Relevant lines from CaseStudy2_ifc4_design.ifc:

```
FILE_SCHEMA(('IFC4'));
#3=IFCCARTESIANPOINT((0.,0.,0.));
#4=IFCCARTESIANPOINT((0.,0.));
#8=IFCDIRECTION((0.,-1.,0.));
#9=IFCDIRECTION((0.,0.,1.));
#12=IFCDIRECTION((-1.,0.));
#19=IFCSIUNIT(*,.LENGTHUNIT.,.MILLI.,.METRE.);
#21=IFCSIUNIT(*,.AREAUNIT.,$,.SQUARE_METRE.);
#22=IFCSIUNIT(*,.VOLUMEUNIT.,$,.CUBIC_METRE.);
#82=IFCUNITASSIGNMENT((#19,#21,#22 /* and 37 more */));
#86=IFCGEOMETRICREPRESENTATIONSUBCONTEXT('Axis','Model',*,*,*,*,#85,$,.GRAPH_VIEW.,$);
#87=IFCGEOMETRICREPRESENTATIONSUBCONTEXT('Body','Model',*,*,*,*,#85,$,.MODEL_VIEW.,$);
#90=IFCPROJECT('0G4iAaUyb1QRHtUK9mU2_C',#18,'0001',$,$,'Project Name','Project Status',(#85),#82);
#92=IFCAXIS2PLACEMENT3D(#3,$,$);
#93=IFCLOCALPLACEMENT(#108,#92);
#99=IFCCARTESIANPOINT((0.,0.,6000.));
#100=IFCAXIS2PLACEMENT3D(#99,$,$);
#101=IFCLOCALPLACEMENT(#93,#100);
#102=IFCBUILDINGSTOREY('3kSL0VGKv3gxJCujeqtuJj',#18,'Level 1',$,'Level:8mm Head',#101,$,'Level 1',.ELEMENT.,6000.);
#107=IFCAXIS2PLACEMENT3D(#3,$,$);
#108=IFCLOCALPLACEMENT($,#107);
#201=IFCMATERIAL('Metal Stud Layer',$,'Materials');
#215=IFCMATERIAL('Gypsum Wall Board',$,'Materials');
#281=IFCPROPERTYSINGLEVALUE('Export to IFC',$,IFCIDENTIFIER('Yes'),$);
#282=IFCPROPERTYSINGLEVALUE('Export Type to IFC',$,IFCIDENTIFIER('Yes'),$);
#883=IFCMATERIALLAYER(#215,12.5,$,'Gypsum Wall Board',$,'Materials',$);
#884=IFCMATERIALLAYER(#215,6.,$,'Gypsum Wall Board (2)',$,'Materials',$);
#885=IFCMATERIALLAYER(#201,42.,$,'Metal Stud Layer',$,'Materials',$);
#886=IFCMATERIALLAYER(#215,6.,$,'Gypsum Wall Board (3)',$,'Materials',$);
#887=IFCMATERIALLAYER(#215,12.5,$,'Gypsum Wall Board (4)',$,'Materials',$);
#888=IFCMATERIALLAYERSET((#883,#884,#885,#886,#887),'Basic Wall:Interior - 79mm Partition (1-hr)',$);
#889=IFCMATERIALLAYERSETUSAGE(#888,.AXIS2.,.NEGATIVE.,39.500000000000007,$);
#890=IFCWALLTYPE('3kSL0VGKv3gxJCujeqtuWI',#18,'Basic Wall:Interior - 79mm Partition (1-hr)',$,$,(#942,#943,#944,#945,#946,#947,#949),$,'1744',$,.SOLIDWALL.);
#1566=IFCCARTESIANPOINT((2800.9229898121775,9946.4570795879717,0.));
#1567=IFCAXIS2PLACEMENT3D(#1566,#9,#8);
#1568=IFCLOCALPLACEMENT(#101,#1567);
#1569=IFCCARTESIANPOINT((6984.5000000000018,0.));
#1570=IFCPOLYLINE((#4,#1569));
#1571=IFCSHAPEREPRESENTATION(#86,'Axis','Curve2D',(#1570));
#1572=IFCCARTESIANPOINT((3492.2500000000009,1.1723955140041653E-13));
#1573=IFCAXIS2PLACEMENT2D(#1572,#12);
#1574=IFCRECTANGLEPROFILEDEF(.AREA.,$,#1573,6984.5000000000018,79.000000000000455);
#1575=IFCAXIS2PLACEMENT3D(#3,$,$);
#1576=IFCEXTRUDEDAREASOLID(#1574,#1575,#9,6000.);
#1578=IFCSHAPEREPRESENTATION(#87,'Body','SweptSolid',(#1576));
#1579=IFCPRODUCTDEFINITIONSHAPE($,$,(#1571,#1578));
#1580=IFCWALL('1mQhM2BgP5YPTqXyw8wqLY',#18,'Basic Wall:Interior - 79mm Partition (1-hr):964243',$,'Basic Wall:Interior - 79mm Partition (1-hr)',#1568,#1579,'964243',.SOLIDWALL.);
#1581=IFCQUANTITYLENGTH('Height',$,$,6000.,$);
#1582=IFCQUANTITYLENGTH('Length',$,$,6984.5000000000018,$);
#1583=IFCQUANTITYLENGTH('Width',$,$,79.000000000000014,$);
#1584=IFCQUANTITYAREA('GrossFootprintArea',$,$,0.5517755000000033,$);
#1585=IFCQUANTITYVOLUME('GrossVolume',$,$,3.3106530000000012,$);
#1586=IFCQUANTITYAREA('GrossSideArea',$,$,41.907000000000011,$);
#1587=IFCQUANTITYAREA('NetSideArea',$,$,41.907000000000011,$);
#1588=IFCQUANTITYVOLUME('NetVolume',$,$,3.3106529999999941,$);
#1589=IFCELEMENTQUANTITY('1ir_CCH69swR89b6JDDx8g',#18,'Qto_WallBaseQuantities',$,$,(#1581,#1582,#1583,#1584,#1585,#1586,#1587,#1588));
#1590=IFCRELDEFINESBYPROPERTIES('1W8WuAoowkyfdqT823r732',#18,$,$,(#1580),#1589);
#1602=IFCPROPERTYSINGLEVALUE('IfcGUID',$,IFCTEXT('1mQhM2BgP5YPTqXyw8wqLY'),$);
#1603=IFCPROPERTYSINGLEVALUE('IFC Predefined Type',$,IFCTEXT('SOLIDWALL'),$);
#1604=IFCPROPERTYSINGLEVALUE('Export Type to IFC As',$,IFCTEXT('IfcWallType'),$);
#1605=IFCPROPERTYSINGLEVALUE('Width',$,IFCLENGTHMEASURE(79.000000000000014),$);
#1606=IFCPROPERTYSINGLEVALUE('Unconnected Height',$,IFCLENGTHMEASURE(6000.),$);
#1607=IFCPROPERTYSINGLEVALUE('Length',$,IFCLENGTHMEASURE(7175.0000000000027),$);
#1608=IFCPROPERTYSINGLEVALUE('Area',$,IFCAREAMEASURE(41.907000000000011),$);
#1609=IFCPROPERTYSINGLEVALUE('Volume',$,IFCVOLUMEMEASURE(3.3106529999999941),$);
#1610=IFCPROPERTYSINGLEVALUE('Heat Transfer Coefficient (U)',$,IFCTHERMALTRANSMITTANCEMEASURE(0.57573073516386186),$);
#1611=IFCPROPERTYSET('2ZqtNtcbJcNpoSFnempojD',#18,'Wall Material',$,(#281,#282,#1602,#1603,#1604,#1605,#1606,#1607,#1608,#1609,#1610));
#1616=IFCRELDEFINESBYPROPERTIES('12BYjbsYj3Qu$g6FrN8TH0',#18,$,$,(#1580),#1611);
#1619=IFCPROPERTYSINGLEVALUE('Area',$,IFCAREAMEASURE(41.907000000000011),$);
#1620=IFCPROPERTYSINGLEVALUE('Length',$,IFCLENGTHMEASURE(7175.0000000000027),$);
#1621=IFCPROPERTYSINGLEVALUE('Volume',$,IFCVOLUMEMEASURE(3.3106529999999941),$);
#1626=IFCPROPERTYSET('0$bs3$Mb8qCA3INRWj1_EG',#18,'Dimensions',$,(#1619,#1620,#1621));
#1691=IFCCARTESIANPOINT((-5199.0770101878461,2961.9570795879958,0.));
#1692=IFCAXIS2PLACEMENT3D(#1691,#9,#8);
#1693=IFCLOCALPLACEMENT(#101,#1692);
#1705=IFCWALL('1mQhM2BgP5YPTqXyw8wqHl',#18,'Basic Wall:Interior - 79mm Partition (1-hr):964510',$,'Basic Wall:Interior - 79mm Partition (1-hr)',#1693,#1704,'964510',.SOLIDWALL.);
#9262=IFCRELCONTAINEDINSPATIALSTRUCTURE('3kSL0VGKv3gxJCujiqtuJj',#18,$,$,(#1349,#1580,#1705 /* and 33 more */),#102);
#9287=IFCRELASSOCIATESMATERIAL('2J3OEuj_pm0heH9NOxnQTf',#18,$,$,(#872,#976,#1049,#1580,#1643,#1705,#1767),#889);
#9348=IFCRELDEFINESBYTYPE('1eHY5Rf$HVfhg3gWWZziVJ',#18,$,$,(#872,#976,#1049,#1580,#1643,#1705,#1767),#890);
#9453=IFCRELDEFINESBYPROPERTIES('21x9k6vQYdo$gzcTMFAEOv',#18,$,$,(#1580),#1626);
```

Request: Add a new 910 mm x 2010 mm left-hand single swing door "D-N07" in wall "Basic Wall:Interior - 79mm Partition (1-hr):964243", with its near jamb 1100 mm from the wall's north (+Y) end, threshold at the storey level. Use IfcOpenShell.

```python
import numpy as np
import ifcopenshell
import ifcopenshell.api.feature
import ifcopenshell.api.geometry
import ifcopenshell.api.pset
import ifcopenshell.api.root
import ifcopenshell.api.spatial
import ifcopenshell.geom
import ifcopenshell.util.element
import ifcopenshell.util.placement
import ifcopenshell.util.representation
import ifcopenshell.util.shape
import ifcopenshell.util.unit

model = ifcopenshell.open("CaseStudy2_ifc4_design.ifc")
unit_scale = ifcopenshell.util.unit.calculate_unit_scale(model)
area_scale = ifcopenshell.util.unit.calculate_unit_scale(model, "AREAUNIT")
volume_scale = ifcopenshell.util.unit.calculate_unit_scale(model, "VOLUMEUNIT")
settings = ifcopenshell.geom.settings()


def volume(element):
    """Net volume in cubic metres, openings subtracted."""
    shape = ifcopenshell.geom.create_shape(settings, element)
    return ifcopenshell.util.shape.get_volume(shape.geometry)


wall = model.by_guid("1mQhM2BgP5YPTqXyw8wqLY")
storey = ifcopenshell.util.element.get_container(wall, ifc_class="IfcBuildingStorey")
context = ifcopenshell.util.representation.get_context(model, "Model", "Body", "MODEL_VIEW")
before = volume(wall)

width, height, from_end, sill = 0.91, 2.01, 1.1, 0.0  # metres

# The wall runs along its own X axis, and the end named is its -X end.
wall_shape = ifcopenshell.geom.create_shape(settings, wall)
x, y, z = ifcopenshell.util.shape.get_vertices(wall_shape.geometry).T
start = x.min() + from_end
face, thickness = float(y.min()), float(y.max() - y.min())
wall_matrix = ifcopenshell.util.placement.get_local_placement(wall.ObjectPlacement)
level = ifcopenshell.util.placement.get_local_placement(storey.ObjectPlacement)[2, 3]


def in_wall(x, y):
    """Placement at x, y metres in the wall's axes, at sill height."""
    matrix = wall_matrix.copy()
    matrix[:, 3] = wall_matrix @ np.array([x / unit_scale, y / unit_scale, 0.0, 1.0])
    matrix[2, 3] = level + sill / unit_scale
    return matrix


# Opening: a box that overshoots both wall faces by 50 mm.
opening = ifcopenshell.api.root.create_entity(model, ifc_class="IfcOpeningElement", predefined_type="OPENING")
box = ifcopenshell.api.geometry.add_wall_representation(
    model, context=context, length=width, height=height, thickness=thickness + 0.1
)
ifcopenshell.api.geometry.assign_representation(model, product=opening, representation=box)
ifcopenshell.api.geometry.edit_object_placement(model, product=opening, matrix=in_wall(start, face - 0.05), is_si=False)
ifcopenshell.api.feature.add_feature(model, feature=opening, element=wall)

door = ifcopenshell.api.root.create_entity(model, ifc_class="IfcDoor", name="D-N07", predefined_type="DOOR")
door.OverallWidth, door.OverallHeight = width / unit_scale, height / unit_scale
door.OperationType = "SINGLE_SWING_LEFT"
body = ifcopenshell.api.geometry.add_door_representation(
    model,
    context=context,
    overall_width=door.OverallWidth,
    overall_height=door.OverallHeight,
    operation_type="SINGLE_SWING_LEFT",
    lining_properties={"LiningDepth": thickness / unit_scale, "ThresholdDepth": thickness / unit_scale},
)
ifcopenshell.api.geometry.assign_representation(model, product=door, representation=body)
ifcopenshell.api.spatial.assign_container(model, products=[door], relating_structure=storey)
ifcopenshell.api.feature.add_filling(model, opening=opening, element=door)

# The lining spans the wall, so the door starts at the wall face.
ifcopenshell.api.geometry.edit_object_placement(model, product=door, matrix=in_wall(start, face), is_si=False)

after = volume(wall)

# Update the wall's stored quantities.
qto = model.by_id(ifcopenshell.util.element.get_pset(wall, "Qto_WallBaseQuantities", should_inherit=False)["id"])
ifcopenshell.api.pset.edit_qto(model, qto=qto, properties={
    "NetSideArea": after / thickness / area_scale,
    "NetVolume": after / volume_scale,
})
pset = model.by_id(ifcopenshell.util.element.get_pset(wall, "Wall Material", should_inherit=False)["id"])
ifcopenshell.api.pset.edit_pset(model, pset=pset, properties={
    "Area": model.create_entity("IfcAreaMeasure", after / thickness / area_scale),
    "Volume": model.create_entity("IfcVolumeMeasure", after / volume_scale),
})
pset = model.by_id(ifcopenshell.util.element.get_pset(wall, "Dimensions", should_inherit=False)["id"])
ifcopenshell.api.pset.edit_pset(model, pset=pset, properties={
    "Area": model.create_entity("IfcAreaMeasure", after / thickness / area_scale),
    "Volume": model.create_entity("IfcVolumeMeasure", after / volume_scale),
})

print(f"wall volume {before:.3f} -> {after:.3f} m3")

model.write("CaseStudy2_ifc4_design_edited.ifc")
```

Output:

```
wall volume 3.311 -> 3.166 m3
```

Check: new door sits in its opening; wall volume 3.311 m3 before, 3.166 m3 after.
